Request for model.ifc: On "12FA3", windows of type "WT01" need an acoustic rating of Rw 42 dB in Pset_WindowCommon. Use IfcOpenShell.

First a look at what the model holds.

```python
import ifcopenshell
import ifcopenshell.util.element

model = ifcopenshell.open("model.ifc")
print(model.schema)
storey = next(s for s in model.by_type("IfcBuildingStorey") if s.Name == "12FA3")
windows = [e for e in ifcopenshell.util.element.get_decomposition(storey) if e.is_a("IfcWindow")]
seen = {}
for e in windows:
    element_type = ifcopenshell.util.element.get_type(e)
    key = (element_type.Name if element_type != e and element_type else None, ifcopenshell.util.element.get_pset(e, "Pset_WindowCommon", "AcousticRating"))
    seen[key] = seen.get(key, 0) + 1
for (name, value), count in sorted(seen.items(), key=str):
    print(count, "x", name, "|", value)
```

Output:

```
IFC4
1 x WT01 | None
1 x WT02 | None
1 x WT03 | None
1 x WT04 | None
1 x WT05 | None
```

```python
import ifcopenshell
import ifcopenshell.api.pset
import ifcopenshell.util.element

model = ifcopenshell.open("model.ifc")

storey = next(s for s in model.by_type("IfcBuildingStorey") if s.Name == "12FA3")
windows = [e for e in ifcopenshell.util.element.get_decomposition(storey) if e.is_a("IfcWindow")]

count = 0
for e in windows:
    element_type = ifcopenshell.util.element.get_type(e)
    if element_type in (None, e) or element_type.Name != "WT01":
        continue
    # add_pset returns the element's existing set when there is one.
    pset = ifcopenshell.api.pset.add_pset(model, product=e, name="Pset_WindowCommon")
    ifcopenshell.api.pset.edit_pset(model, pset=pset, properties={"AcousticRating": "Rw 42 dB"})
    count += 1

print(count, "windows updated")

model.write("model_edited.ifc")
```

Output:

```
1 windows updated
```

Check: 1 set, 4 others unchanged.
